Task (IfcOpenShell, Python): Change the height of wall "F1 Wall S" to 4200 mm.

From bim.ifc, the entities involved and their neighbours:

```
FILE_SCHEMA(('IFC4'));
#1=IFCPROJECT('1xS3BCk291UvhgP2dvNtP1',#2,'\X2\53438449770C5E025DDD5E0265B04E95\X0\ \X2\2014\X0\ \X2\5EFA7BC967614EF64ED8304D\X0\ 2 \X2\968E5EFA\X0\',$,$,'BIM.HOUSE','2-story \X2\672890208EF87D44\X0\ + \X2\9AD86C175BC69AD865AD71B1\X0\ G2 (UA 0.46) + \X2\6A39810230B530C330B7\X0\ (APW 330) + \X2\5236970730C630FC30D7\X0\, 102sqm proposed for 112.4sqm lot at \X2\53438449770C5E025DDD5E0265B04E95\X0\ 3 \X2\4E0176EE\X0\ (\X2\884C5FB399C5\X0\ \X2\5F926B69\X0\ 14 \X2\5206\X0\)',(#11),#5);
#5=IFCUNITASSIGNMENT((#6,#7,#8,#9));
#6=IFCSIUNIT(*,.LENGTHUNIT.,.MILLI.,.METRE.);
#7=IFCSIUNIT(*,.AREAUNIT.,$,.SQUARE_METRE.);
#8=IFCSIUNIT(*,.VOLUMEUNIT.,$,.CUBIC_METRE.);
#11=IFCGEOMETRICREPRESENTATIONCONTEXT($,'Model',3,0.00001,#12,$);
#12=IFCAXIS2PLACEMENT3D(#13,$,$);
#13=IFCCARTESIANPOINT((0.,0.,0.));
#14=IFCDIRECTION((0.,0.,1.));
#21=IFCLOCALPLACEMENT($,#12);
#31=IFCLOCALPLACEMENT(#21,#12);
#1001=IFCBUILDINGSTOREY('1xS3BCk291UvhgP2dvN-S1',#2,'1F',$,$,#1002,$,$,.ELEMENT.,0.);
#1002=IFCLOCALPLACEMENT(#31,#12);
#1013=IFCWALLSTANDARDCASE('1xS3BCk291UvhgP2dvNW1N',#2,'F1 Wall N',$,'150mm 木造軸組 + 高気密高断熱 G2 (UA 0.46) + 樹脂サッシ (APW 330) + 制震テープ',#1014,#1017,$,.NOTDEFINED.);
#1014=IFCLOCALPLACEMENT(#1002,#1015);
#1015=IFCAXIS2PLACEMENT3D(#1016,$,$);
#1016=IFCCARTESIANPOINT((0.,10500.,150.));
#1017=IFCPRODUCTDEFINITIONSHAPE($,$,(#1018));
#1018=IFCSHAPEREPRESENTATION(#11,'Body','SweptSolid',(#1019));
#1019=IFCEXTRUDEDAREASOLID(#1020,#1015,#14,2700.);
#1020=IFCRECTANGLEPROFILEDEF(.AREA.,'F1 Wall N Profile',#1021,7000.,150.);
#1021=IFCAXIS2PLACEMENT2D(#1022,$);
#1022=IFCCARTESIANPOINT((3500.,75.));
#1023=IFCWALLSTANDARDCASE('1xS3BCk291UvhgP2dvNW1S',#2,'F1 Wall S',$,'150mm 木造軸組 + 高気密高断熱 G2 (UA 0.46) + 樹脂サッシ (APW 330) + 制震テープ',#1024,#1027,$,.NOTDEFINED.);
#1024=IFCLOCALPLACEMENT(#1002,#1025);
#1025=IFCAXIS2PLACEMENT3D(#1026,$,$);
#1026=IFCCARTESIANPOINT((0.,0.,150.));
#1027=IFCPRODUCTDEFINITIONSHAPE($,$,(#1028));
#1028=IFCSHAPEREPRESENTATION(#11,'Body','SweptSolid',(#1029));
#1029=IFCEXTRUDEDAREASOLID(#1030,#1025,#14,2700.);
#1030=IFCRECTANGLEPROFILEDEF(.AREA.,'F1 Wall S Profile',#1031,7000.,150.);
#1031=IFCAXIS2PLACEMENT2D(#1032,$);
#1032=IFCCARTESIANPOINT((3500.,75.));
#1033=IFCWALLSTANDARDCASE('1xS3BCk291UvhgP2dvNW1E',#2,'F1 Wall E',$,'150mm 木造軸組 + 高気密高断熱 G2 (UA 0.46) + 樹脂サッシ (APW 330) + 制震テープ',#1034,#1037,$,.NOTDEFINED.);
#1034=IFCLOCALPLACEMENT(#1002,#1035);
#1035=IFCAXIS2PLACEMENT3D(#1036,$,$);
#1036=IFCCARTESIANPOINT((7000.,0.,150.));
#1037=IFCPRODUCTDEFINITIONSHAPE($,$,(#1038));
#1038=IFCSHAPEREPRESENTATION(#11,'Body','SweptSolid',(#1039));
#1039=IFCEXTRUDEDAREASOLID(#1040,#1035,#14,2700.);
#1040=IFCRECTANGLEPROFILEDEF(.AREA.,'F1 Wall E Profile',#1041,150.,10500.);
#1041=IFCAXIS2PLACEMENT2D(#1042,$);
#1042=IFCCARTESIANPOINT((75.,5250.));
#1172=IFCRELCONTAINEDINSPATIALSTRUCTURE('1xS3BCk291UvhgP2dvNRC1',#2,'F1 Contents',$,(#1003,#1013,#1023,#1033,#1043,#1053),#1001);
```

```python
import ifcopenshell
import ifcopenshell.geom
import ifcopenshell.util.shape
import ifcopenshell.util.unit

model = ifcopenshell.open("bim.ifc")
unit_scale = ifcopenshell.util.unit.calculate_unit_scale(model)
settings = ifcopenshell.geom.settings()


def volume(element):
    """Net volume in cubic metres, openings subtracted."""
    shape = ifcopenshell.geom.create_shape(settings, element)
    return ifcopenshell.util.shape.get_volume(shape.geometry)


wall = model.by_guid("1xS3BCk291UvhgP2dvNW1S")
before = volume(wall)

body = next(r for r in wall.Representation.Representations if r.RepresentationIdentifier == "Body")
solid = body.Items[0]
old_height = solid.Depth
solid.Depth = 4.2 / unit_scale
after = volume(wall)

print(f"height {old_height:g} -> {solid.Depth:g}, volume {before:.3f} -> {after:.3f} m3")

model.write("bim-out.ifc")
```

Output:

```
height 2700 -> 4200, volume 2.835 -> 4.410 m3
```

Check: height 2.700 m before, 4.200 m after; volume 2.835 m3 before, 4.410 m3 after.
